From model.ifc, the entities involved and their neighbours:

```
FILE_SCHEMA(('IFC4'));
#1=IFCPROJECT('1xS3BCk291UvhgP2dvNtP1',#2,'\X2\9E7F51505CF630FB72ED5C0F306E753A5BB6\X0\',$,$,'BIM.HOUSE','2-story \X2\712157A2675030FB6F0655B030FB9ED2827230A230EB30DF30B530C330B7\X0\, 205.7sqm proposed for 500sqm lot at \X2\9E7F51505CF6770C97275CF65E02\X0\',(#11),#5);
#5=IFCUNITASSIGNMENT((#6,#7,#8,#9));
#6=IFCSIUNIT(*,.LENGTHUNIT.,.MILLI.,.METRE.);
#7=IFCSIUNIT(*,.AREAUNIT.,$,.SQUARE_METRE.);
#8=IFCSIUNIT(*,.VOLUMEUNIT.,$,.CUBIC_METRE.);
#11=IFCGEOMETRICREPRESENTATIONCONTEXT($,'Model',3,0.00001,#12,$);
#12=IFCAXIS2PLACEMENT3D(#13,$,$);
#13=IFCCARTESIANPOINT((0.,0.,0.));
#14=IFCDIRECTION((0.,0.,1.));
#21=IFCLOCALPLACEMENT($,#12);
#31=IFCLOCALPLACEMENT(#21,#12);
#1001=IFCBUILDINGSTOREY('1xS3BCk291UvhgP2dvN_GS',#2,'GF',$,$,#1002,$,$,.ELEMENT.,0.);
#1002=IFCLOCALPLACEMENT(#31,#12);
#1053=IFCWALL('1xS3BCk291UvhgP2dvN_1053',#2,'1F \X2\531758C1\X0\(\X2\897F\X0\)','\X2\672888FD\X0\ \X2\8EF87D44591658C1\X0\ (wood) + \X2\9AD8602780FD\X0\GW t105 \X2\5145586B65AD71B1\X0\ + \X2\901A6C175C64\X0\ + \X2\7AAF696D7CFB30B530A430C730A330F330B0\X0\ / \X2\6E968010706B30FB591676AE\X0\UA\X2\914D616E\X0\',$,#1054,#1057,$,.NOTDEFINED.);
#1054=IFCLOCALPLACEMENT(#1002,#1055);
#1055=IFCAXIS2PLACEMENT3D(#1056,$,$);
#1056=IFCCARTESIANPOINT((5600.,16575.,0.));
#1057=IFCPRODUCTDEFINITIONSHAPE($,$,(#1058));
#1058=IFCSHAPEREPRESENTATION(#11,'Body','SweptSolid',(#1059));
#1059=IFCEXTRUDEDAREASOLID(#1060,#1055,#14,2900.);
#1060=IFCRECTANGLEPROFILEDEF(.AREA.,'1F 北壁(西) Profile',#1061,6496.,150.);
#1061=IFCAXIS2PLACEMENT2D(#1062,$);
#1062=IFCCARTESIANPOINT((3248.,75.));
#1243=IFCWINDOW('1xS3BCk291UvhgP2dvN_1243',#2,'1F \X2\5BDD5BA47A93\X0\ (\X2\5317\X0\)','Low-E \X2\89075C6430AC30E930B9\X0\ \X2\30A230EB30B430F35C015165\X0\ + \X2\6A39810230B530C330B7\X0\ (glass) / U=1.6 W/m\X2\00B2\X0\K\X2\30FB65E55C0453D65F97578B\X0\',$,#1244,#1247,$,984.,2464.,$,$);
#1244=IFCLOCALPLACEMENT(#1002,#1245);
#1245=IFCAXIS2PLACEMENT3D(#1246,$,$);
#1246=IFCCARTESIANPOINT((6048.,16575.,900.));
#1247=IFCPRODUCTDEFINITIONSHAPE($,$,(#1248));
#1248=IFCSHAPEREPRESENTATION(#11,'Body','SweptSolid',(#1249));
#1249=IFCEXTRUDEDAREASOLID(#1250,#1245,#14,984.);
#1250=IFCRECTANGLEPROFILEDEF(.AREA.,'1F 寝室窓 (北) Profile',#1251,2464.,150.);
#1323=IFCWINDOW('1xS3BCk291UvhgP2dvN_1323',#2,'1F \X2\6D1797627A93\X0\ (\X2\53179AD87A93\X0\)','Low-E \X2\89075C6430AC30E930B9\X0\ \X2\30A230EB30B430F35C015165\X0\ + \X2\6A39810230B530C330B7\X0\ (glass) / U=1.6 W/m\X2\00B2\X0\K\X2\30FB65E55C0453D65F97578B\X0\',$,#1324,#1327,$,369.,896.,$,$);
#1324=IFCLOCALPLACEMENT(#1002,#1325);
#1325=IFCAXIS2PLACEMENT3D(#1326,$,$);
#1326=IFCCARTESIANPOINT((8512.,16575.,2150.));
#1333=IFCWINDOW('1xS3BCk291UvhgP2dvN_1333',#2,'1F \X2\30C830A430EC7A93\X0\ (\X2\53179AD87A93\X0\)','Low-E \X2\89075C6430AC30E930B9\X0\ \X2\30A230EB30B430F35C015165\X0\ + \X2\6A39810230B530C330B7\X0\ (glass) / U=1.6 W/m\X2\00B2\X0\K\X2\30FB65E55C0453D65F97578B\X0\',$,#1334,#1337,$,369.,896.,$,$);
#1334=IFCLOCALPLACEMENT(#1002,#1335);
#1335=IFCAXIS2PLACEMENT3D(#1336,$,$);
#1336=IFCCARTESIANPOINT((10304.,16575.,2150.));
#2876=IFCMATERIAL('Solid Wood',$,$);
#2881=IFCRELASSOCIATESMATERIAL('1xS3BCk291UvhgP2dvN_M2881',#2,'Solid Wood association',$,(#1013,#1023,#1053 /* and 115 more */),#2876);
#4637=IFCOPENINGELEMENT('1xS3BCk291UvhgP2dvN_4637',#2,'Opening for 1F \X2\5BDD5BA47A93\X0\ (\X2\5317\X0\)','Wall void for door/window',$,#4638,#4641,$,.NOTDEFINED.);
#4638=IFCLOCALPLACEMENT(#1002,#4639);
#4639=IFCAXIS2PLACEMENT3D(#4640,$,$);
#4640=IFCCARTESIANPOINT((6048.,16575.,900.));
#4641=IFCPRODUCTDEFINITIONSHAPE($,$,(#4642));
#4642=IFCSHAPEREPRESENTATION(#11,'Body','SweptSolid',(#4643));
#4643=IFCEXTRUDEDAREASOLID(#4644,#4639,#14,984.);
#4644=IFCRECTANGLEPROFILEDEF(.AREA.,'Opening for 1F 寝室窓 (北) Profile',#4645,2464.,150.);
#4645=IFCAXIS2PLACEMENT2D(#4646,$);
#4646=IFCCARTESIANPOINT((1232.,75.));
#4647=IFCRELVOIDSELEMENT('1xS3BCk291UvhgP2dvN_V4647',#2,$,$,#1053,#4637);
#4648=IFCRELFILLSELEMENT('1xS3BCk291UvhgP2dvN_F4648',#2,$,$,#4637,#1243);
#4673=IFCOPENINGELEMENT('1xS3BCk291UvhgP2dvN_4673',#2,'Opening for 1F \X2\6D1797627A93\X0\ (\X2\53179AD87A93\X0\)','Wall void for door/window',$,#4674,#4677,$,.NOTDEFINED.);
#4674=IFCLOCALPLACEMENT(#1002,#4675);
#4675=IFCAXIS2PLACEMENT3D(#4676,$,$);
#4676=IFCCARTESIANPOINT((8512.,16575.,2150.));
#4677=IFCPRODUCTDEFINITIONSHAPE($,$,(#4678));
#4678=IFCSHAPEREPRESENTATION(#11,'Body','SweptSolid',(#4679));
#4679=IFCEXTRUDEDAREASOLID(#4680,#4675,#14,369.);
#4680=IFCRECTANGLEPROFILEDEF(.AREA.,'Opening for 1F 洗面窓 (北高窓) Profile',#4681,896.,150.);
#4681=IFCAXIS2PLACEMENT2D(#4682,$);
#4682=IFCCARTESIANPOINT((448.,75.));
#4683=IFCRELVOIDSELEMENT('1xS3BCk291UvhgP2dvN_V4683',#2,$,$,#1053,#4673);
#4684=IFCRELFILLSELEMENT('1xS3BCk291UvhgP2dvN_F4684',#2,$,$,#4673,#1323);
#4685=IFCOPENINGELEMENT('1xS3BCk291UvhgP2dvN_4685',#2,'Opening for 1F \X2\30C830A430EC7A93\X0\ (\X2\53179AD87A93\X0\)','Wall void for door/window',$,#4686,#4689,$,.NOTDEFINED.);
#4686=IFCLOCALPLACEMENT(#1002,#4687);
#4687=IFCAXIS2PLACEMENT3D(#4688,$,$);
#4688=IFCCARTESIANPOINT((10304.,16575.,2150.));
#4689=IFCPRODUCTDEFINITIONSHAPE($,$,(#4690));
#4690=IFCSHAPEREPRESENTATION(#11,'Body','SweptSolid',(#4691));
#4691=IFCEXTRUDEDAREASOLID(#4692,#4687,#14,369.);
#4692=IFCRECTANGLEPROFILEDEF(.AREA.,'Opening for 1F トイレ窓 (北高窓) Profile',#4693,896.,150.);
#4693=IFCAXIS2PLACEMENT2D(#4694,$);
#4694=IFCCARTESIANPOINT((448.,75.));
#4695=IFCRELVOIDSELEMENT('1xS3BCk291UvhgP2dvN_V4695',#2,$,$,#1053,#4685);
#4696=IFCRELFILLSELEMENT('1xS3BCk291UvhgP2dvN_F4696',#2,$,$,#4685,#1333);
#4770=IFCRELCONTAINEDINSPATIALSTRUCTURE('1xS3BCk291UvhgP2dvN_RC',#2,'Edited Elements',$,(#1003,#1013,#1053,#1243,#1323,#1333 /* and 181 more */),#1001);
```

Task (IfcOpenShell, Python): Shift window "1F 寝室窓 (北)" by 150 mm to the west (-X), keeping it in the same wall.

```python
import ifcopenshell
import ifcopenshell.api.geometry
import ifcopenshell.util.placement
import ifcopenshell.util.unit

model = ifcopenshell.open("model.ifc")
unit_scale = ifcopenshell.util.unit.calculate_unit_scale(model)

window = model.by_guid("1xS3BCk291UvhgP2dvN_1243")
opening = window.FillsVoids[0].RelatingOpeningElement
wall = opening.VoidsElements[0].RelatingBuildingElement

wall_matrix = ifcopenshell.util.placement.get_local_placement(wall.ObjectPlacement)
shift = wall_matrix[:3, 0] * -0.15 / unit_scale
before = ifcopenshell.util.placement.get_local_placement(window.ObjectPlacement)[:3, 3].copy()

# The window is not placed relative to its opening, so move both.
for product in (opening, window):
    matrix = ifcopenshell.util.placement.get_local_placement(product.ObjectPlacement)
    matrix[:3, 3] += shift
    ifcopenshell.api.geometry.edit_object_placement(model, product=product, matrix=matrix, is_si=False)

after = ifcopenshell.util.placement.get_local_placement(window.ObjectPlacement)[:3, 3]
print("window moved by", (after - before).round(3) + 0.0)

model.write("model_updated.ifc")
```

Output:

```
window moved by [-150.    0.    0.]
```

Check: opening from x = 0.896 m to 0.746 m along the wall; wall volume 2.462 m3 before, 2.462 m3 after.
